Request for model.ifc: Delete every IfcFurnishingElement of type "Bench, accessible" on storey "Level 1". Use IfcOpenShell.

First a look at what the model holds.

```python
import ifcopenshell
import ifcopenshell.util.element

model = ifcopenshell.open("model.ifc")
print(model.schema)
storey = next(s for s in model.by_type("IfcBuildingStorey") if s.Name == "Level 1")
furniture = [e for e in ifcopenshell.util.element.get_decomposition(storey) if e.is_a("IfcFurnishingElement")]
seen = {}
for e in furniture:
    element_type = ifcopenshell.util.element.get_type(e)
    name = element_type.Name if element_type not in (None, e) else None
    seen[name] = seen.get(name, 0) + 1
for name, count in sorted(seen.items(), key=str):
    print(count, "x", name)
```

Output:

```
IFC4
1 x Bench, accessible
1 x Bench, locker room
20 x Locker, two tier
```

```python
import ifcopenshell
import ifcopenshell.api.root
import ifcopenshell.util.element

model = ifcopenshell.open("model.ifc")

storey = next(s for s in model.by_type("IfcBuildingStorey") if s.Name == "Level 1")
furniture = [e for e in ifcopenshell.util.element.get_decomposition(storey) if e.is_a("IfcFurnishingElement")]
targets = [e for e in furniture if (t := ifcopenshell.util.element.get_type(e)) not in (None, e) and t.Name == "Bench, accessible"]

for e in targets:
    ifcopenshell.api.root.remove_product(model, product=e)
print(len(targets), "removed")

model.write("model_updated.ifc")
```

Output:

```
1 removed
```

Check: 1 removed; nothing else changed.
